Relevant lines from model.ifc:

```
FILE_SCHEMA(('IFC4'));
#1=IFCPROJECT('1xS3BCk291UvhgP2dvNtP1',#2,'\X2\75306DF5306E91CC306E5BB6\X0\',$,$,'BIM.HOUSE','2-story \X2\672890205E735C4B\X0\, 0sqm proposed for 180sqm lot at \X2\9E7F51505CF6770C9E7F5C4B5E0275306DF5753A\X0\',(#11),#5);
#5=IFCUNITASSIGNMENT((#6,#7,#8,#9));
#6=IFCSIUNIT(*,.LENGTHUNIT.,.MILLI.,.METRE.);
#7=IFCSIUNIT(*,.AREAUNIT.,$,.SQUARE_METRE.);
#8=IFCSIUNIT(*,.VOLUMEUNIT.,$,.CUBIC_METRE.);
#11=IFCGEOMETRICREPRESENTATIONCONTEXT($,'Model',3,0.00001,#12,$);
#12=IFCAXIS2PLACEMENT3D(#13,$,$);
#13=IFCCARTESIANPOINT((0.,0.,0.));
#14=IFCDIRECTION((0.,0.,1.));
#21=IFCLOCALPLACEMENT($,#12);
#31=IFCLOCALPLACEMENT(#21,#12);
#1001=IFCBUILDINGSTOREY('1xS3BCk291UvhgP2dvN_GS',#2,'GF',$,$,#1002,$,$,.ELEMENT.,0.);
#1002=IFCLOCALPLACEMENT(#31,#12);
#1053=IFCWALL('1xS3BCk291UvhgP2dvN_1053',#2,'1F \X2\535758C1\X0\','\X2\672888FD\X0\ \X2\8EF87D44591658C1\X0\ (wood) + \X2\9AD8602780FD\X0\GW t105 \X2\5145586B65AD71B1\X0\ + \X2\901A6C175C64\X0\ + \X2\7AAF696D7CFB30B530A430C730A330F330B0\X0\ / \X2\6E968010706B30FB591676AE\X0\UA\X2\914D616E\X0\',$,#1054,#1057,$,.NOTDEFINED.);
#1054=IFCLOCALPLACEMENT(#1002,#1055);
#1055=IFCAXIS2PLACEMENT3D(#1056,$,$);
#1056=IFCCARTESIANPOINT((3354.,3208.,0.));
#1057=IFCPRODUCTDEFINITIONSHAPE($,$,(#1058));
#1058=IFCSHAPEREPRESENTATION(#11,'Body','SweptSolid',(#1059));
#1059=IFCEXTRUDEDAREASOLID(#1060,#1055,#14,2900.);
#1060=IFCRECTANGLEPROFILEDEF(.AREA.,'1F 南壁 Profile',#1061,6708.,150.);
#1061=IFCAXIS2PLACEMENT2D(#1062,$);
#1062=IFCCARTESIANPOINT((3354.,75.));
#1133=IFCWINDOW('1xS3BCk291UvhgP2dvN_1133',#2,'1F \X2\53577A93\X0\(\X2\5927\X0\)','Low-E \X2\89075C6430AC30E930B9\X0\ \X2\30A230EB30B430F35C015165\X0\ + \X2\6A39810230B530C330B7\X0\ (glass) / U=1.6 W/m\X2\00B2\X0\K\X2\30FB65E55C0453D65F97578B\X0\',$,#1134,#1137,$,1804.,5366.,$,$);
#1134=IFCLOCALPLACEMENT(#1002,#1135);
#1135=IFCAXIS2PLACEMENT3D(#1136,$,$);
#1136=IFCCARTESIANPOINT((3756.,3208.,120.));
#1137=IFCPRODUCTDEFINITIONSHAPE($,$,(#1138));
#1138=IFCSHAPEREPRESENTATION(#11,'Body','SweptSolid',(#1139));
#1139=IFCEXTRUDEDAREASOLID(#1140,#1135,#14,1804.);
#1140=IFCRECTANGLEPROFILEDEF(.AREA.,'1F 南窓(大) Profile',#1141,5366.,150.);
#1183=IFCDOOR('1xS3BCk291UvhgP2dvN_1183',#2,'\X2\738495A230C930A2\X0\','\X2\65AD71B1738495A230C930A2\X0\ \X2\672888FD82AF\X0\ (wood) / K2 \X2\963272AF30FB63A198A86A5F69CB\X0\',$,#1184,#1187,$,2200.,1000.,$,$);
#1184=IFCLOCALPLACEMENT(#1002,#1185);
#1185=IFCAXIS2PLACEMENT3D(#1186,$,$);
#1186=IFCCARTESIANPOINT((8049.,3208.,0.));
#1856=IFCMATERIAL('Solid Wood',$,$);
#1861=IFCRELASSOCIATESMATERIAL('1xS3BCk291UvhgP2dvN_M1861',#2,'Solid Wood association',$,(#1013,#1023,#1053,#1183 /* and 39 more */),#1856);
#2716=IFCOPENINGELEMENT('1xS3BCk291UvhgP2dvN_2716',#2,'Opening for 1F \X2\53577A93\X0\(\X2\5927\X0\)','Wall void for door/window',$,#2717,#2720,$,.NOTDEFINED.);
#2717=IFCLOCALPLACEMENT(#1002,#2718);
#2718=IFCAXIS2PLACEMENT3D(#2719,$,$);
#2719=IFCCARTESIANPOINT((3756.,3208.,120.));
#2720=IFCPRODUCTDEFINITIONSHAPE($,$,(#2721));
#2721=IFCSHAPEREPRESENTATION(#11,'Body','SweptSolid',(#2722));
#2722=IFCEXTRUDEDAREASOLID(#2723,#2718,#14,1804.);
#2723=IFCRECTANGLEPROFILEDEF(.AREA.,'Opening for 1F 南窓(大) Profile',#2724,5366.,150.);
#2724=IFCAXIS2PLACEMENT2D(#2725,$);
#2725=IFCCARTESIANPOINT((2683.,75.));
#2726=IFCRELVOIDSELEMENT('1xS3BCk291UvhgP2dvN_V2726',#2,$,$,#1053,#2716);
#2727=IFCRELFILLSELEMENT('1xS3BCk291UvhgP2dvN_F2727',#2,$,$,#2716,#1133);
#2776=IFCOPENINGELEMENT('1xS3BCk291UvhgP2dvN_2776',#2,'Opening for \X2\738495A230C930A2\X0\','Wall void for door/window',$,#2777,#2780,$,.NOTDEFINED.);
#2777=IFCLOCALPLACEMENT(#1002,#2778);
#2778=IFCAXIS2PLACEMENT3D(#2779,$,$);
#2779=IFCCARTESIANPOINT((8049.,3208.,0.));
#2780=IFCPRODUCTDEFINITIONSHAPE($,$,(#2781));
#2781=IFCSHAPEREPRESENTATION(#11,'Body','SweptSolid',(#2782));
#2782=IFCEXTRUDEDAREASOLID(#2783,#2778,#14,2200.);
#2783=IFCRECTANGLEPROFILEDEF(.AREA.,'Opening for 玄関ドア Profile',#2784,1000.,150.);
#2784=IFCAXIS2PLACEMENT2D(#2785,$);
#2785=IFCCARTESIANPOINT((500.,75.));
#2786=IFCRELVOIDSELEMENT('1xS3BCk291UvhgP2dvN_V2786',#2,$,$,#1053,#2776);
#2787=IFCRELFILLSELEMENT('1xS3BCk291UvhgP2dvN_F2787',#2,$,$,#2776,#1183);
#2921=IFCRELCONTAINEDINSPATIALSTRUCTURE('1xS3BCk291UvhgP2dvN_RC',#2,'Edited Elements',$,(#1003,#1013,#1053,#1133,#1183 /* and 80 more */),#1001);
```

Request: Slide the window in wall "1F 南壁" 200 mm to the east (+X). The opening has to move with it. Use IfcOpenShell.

```python
import ifcopenshell
import ifcopenshell.api.geometry
import ifcopenshell.util.placement

model = ifcopenshell.open("model.ifc")

window = model.by_id(1133)
opening = window.FillsVoids[0].RelatingOpeningElement
wall = opening.VoidsElements[0].RelatingBuildingElement

wall_matrix = ifcopenshell.util.placement.get_local_placement(wall.ObjectPlacement)
shift = wall_matrix[:3, 0] * 200.0
before = ifcopenshell.util.placement.get_local_placement(window.ObjectPlacement)[:3, 3].copy()

# The window is not placed relative to its opening, so move both.
for product in (opening, window):
    matrix = ifcopenshell.util.placement.get_local_placement(product.ObjectPlacement)
    matrix[:3, 3] += shift
    ifcopenshell.api.geometry.edit_object_placement(model, product=product, matrix=matrix, is_si=False)

after = ifcopenshell.util.placement.get_local_placement(window.ObjectPlacement)[:3, 3]
print("window moved by", (after - before).round(3) + 0.0)

model.write("model_rev.ifc")
```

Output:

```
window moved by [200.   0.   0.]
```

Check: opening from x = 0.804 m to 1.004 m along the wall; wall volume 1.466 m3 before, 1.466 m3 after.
